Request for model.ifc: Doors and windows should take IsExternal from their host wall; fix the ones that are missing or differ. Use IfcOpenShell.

First a look at what the model holds.

```python
import ifcopenshell
import ifcopenshell.util.element

model = ifcopenshell.open("model.ifc")
print(model.schema)
seen = {}
for e in model.by_type("IfcDoor") + model.by_type("IfcWindow"):
    if not e.FillsVoids:
        continue
    host = e.FillsVoids[0].RelatingOpeningElement.VoidsElements[0].RelatingBuildingElement
    own = ifcopenshell.util.element.get_pset(e, f"Pset_{e.is_a()[3:].removesuffix('StandardCase')}Common", "IsExternal")
    wall = ifcopenshell.util.element.get_pset(host, "Pset_WallCommon", "IsExternal")
    seen[e.is_a(), own, wall] = seen.get((e.is_a(), own, wall), 0) + 1
for (cls, own, wall), count in sorted(seen.items(), key=str):
    print(count, cls, "IsExternal:", own, "| host wall:", wall)
```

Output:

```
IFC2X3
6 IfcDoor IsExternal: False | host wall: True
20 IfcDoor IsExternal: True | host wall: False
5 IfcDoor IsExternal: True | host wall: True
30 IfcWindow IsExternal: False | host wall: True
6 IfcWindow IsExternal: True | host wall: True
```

```python
import ifcopenshell
import ifcopenshell.api.pset
import ifcopenshell.util.element

model = ifcopenshell.open("model.ifc")

count = 0
for ifc_class, pset_name in (("IfcDoor", "Pset_DoorCommon"), ("IfcWindow", "Pset_WindowCommon")):
    for e in model.by_type(ifc_class):
        if not e.FillsVoids:
            continue
        host = e.FillsVoids[0].RelatingOpeningElement.VoidsElements[0].RelatingBuildingElement
        external = ifcopenshell.util.element.get_pset(host, "Pset_WallCommon", "IsExternal")
        if external is None or ifcopenshell.util.element.get_pset(e, pset_name, "IsExternal") == external:
            continue
        pset = ifcopenshell.api.pset.add_pset(model, product=e, name=pset_name)
        ifcopenshell.api.pset.edit_pset(model, pset=pset, properties={"IsExternal": external})
        count += 1

print(count, "updated")

model.write("model_updated.ifc")
```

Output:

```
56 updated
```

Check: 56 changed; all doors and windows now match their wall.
